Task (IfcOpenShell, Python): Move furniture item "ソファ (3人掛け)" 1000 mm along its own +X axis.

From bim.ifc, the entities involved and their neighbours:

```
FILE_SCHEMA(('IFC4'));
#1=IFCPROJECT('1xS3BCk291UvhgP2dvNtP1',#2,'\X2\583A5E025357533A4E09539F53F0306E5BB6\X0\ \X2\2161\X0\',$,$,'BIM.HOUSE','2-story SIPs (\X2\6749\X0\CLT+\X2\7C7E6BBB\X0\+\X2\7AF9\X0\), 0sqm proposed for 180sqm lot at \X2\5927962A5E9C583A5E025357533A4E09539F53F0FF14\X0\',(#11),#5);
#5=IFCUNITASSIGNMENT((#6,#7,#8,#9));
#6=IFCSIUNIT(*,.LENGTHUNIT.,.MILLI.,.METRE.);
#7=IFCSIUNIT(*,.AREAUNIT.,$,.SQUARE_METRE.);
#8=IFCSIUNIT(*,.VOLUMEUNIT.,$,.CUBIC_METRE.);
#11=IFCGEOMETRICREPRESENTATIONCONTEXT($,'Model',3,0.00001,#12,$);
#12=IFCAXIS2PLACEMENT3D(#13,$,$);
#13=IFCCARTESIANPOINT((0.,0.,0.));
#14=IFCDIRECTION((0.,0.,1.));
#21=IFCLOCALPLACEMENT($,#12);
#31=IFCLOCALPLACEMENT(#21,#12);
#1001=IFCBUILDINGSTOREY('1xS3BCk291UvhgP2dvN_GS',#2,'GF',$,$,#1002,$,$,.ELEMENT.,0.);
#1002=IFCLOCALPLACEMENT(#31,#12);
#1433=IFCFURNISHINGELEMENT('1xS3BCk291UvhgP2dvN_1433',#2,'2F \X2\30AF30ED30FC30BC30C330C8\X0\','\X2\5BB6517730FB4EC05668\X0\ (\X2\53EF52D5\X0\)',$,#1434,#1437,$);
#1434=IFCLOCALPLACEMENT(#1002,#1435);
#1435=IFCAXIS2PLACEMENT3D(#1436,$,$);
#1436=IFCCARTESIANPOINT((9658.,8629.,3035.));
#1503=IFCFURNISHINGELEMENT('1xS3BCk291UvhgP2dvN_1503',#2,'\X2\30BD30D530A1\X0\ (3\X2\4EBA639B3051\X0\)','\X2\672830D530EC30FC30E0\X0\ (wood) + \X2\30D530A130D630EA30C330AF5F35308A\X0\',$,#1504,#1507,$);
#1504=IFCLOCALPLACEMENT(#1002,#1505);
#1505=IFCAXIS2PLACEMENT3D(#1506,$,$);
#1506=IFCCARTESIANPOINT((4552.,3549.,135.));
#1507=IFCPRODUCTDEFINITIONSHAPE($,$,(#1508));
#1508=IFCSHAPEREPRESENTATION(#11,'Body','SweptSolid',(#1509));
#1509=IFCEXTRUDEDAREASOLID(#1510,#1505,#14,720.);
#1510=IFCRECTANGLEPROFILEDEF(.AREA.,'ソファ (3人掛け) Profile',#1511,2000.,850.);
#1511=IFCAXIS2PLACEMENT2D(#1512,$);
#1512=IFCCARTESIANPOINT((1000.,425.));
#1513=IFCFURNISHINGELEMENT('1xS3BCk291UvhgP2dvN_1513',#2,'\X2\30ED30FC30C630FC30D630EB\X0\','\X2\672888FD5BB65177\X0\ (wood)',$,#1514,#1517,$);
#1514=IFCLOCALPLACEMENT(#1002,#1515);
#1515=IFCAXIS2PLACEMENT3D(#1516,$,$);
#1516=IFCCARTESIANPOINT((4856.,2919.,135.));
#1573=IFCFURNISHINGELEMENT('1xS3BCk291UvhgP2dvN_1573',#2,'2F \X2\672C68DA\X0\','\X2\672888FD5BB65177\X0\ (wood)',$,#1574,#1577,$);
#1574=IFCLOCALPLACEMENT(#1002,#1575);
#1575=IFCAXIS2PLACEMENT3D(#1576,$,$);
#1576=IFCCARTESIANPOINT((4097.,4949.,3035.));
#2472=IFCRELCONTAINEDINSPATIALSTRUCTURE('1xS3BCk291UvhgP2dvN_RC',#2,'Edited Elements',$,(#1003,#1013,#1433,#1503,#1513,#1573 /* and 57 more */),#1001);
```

```python
import ifcopenshell
import ifcopenshell.api.geometry
import ifcopenshell.util.placement
import ifcopenshell.util.unit

model = ifcopenshell.open("bim.ifc")
unit_scale = ifcopenshell.util.unit.calculate_unit_scale(model)

item = model.by_id(1503)
matrix = ifcopenshell.util.placement.get_local_placement(item.ObjectPlacement)
matrix[:3, 3] += matrix[:3, 0] * 1 / unit_scale
ifcopenshell.api.geometry.edit_object_placement(model, product=item, matrix=matrix, is_si=False)

print(ifcopenshell.util.placement.get_local_placement(item.ObjectPlacement).round(3) + 0.0)

model.write("bim_v2.ifc")
```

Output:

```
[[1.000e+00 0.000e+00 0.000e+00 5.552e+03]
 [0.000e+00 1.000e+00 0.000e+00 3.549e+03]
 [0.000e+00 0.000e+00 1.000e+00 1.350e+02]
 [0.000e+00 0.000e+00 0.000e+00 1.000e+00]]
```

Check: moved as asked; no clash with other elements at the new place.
